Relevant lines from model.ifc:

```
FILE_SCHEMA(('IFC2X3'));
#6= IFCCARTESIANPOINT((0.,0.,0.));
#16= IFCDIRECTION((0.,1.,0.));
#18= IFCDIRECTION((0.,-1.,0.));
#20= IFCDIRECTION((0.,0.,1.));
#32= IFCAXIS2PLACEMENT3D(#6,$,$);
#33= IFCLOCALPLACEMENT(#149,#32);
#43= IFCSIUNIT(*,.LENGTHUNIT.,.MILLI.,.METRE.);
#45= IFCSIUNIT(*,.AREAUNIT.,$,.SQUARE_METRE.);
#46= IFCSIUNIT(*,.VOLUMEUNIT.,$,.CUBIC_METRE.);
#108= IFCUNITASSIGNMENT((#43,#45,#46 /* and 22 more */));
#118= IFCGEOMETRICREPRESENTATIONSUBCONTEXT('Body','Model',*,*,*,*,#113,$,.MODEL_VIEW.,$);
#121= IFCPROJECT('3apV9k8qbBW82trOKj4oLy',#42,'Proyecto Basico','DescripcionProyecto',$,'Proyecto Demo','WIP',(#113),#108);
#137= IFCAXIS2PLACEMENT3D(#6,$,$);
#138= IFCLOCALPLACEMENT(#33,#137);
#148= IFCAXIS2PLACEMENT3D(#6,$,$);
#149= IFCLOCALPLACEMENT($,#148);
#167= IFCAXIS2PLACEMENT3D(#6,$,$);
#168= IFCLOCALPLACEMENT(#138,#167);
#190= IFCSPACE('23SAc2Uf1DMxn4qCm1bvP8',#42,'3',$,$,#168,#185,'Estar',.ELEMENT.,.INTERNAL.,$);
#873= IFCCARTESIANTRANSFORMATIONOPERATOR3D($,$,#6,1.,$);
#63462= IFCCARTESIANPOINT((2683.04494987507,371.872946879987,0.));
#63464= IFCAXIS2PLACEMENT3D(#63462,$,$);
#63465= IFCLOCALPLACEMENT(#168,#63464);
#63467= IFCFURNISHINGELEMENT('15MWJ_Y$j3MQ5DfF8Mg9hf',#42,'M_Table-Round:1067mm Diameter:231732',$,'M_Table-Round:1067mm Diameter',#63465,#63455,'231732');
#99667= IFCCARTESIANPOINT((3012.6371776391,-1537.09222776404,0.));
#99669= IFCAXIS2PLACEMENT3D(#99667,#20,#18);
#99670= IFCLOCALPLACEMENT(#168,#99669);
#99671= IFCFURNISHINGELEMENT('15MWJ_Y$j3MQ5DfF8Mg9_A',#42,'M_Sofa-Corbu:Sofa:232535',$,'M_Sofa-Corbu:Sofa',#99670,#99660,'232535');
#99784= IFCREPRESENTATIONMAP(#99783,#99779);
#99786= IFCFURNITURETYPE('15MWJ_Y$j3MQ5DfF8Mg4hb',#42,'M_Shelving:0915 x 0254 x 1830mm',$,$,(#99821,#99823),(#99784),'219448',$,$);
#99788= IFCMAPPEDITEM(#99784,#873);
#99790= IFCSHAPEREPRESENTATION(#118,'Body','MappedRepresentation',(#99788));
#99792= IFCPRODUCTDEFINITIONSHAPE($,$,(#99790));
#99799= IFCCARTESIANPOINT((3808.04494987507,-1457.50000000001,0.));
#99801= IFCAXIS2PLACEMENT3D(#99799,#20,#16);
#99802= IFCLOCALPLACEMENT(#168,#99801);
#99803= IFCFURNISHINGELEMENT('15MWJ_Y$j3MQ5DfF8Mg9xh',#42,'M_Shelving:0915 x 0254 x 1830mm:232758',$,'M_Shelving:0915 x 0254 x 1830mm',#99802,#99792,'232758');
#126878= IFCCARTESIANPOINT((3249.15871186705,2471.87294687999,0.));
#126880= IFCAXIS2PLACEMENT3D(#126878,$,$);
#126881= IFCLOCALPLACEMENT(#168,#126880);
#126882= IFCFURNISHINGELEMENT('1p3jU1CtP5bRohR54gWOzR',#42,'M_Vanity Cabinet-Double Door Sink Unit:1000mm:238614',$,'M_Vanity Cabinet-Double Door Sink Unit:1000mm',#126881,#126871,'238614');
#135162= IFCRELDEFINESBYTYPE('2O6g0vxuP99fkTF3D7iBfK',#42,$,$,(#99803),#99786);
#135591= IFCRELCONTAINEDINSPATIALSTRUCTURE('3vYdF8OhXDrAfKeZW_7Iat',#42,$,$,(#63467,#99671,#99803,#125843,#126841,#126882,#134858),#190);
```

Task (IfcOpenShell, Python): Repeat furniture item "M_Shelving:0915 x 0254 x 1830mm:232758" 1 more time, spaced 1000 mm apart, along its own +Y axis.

```python
import ifcopenshell
import ifcopenshell.api.geometry
import ifcopenshell.api.root
import ifcopenshell.util.element
import ifcopenshell.util.placement
import ifcopenshell.util.unit

model = ifcopenshell.open("model.ifc")
unit_scale = ifcopenshell.util.unit.calculate_unit_scale(model)


def reuse_history(source, copy):
    """copy_class also copies each property set's owner history, people and application; keep the originals."""
    for rel in copy.IsDefinedBy:
        if rel.is_a("IfcRelDefinesByProperties") and (history := rel.RelatingPropertyDefinition.OwnerHistory):
            rel.RelatingPropertyDefinition.OwnerHistory = source.OwnerHistory
            ifcopenshell.util.element.remove_deep2(model, history)


source = model.by_guid("15MWJ_Y$j3MQ5DfF8Mg9xh")
base = ifcopenshell.util.placement.get_local_placement(source.ObjectPlacement)
step = base[:3, 1] * 1 / unit_scale

for i in range(1, 2):
    copy = ifcopenshell.api.root.copy_class(model, product=source)
    copy.Representation = ifcopenshell.util.element.copy_deep(
        model, source.Representation, exclude=["IfcGeometricRepresentationContext", "IfcRepresentationMap"]
    )
    copy.Name = "M_Shelving:0915 x 0254 x 1830mm"
    copy.Tag = None
    reuse_history(source, copy)
    matrix = base.copy()
    matrix[:3, 3] += i * step
    print("added at", matrix[:3, 3].round(3) + 0.0)
    ifcopenshell.api.geometry.edit_object_placement(model, product=copy, matrix=matrix, is_si=False)

model.write("model_rev.ifc")
```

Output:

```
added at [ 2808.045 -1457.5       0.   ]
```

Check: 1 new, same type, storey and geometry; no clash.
